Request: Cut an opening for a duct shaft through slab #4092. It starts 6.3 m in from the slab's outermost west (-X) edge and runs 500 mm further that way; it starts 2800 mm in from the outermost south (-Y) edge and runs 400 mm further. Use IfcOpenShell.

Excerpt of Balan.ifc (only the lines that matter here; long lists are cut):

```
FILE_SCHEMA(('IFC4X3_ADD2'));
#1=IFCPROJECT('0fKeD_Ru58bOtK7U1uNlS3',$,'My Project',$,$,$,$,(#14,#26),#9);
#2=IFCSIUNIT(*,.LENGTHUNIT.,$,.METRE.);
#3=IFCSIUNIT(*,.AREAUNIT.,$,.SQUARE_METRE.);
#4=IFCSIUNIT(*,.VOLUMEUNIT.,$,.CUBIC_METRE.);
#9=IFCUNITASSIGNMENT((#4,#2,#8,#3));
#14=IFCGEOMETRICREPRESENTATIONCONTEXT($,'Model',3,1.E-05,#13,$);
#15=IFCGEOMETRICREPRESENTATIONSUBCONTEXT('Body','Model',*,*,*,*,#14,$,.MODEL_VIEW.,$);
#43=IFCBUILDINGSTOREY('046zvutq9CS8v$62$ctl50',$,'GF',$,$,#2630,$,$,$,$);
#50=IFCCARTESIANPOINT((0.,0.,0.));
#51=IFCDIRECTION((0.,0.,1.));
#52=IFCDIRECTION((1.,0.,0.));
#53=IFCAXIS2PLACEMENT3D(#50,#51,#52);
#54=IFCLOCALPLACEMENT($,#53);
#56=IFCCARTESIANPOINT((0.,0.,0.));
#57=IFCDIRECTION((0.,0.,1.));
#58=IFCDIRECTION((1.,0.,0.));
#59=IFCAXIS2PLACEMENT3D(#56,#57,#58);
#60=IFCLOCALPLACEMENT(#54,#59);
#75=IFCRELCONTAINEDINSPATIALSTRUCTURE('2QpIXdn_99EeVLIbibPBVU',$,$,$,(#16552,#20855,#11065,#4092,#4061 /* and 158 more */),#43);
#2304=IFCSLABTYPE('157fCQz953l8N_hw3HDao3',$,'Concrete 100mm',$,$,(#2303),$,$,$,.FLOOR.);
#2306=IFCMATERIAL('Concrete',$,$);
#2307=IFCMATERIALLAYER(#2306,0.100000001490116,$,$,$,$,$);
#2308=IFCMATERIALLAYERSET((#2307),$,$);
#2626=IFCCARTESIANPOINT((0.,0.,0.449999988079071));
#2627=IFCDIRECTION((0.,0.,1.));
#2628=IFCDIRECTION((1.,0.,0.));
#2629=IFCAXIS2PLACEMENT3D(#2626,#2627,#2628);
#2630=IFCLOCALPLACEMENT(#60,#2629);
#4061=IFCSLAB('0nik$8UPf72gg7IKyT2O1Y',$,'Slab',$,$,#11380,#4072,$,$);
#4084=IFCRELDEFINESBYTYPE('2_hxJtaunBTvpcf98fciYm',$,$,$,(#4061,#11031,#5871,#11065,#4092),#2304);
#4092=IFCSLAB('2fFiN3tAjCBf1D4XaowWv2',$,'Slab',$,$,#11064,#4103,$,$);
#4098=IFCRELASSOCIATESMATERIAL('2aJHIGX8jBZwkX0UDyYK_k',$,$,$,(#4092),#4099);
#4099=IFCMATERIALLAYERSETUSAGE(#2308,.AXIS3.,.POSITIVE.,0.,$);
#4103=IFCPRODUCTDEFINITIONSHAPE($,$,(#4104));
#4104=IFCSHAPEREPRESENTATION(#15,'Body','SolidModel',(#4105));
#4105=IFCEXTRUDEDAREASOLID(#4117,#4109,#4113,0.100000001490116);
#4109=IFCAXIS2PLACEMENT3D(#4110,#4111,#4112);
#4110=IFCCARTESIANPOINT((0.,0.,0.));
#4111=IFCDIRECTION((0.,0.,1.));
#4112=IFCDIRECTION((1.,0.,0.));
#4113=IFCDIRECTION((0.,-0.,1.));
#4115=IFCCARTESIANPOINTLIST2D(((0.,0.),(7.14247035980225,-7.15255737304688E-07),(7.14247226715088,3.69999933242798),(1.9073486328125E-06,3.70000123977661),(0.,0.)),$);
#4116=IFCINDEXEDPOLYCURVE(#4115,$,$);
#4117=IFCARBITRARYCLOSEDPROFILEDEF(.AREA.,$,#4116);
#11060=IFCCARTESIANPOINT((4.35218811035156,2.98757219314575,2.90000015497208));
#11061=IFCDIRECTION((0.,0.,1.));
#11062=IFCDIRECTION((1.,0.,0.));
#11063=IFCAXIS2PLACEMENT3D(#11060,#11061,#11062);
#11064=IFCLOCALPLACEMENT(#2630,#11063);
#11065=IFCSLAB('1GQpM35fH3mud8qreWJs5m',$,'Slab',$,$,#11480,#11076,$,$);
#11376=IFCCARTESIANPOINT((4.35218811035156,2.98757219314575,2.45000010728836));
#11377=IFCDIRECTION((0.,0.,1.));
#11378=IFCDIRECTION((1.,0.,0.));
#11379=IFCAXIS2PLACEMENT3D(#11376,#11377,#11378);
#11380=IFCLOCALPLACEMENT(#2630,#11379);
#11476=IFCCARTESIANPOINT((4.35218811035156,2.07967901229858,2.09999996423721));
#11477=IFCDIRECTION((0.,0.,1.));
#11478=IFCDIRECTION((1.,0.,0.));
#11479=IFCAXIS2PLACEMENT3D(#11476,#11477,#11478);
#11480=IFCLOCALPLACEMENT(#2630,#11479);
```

```python
import numpy as np
import ifcopenshell
import ifcopenshell.api.feature
import ifcopenshell.api.geometry
import ifcopenshell.api.root
import ifcopenshell.geom
import ifcopenshell.util.placement
import ifcopenshell.util.representation
import ifcopenshell.util.shape
import ifcopenshell.util.unit

model = ifcopenshell.open("Balan.ifc")
unit_scale = ifcopenshell.util.unit.calculate_unit_scale(model)
settings = ifcopenshell.geom.settings()


def volume(element):
    """Net volume in cubic metres, openings subtracted."""
    shape = ifcopenshell.geom.create_shape(settings, element)
    return ifcopenshell.util.shape.get_volume(shape.geometry)


slab = model.by_guid("2fFiN3tAjCBf1D4XaowWv2")
before = volume(slab)

# Extent in the slab's own axes, in metres. The edges named are its -X and -Y sides.
slab_shape = ifcopenshell.geom.create_shape(settings, slab)
vertices = ifcopenshell.util.shape.get_vertices(slab_shape.geometry)
x_min, y_min, bottom = vertices.min(axis=0)
top = vertices[:, 2].max()

opening = ifcopenshell.api.root.create_entity(model, ifc_class="IfcOpeningElement", name="Duct shaft opening", predefined_type="OPENING")
context = ifcopenshell.util.representation.get_context(model, "Model", "Body", "MODEL_VIEW")
width, depth = 0.5, 0.4
outline = [(0.0, 0.0), (width, 0.0), (width, depth), (0.0, depth), (0.0, 0.0)]
# Overshoot both faces by 50 mm so the cut is clean.
shape = ifcopenshell.api.geometry.add_slab_representation(
    model, context=context, depth=top - bottom + 0.1, polyline=outline
)
ifcopenshell.api.geometry.assign_representation(model, product=opening, representation=shape)

matrix = ifcopenshell.util.placement.get_local_placement(slab.ObjectPlacement)
matrix[:, 3] = matrix @ np.append(np.array([x_min + 6.3, y_min + 2.8, bottom - 0.05]) / unit_scale, 1.0)
ifcopenshell.api.geometry.edit_object_placement(model, product=opening, matrix=matrix, is_si=False)
ifcopenshell.api.feature.add_feature(model, feature=opening, element=slab)

after = volume(slab)

print(f"slab volume {before:.3f} -> {after:.3f} m3")

model.write("Balan_v2.ifc")
```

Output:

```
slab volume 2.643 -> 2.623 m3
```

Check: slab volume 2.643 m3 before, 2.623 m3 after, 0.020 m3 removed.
